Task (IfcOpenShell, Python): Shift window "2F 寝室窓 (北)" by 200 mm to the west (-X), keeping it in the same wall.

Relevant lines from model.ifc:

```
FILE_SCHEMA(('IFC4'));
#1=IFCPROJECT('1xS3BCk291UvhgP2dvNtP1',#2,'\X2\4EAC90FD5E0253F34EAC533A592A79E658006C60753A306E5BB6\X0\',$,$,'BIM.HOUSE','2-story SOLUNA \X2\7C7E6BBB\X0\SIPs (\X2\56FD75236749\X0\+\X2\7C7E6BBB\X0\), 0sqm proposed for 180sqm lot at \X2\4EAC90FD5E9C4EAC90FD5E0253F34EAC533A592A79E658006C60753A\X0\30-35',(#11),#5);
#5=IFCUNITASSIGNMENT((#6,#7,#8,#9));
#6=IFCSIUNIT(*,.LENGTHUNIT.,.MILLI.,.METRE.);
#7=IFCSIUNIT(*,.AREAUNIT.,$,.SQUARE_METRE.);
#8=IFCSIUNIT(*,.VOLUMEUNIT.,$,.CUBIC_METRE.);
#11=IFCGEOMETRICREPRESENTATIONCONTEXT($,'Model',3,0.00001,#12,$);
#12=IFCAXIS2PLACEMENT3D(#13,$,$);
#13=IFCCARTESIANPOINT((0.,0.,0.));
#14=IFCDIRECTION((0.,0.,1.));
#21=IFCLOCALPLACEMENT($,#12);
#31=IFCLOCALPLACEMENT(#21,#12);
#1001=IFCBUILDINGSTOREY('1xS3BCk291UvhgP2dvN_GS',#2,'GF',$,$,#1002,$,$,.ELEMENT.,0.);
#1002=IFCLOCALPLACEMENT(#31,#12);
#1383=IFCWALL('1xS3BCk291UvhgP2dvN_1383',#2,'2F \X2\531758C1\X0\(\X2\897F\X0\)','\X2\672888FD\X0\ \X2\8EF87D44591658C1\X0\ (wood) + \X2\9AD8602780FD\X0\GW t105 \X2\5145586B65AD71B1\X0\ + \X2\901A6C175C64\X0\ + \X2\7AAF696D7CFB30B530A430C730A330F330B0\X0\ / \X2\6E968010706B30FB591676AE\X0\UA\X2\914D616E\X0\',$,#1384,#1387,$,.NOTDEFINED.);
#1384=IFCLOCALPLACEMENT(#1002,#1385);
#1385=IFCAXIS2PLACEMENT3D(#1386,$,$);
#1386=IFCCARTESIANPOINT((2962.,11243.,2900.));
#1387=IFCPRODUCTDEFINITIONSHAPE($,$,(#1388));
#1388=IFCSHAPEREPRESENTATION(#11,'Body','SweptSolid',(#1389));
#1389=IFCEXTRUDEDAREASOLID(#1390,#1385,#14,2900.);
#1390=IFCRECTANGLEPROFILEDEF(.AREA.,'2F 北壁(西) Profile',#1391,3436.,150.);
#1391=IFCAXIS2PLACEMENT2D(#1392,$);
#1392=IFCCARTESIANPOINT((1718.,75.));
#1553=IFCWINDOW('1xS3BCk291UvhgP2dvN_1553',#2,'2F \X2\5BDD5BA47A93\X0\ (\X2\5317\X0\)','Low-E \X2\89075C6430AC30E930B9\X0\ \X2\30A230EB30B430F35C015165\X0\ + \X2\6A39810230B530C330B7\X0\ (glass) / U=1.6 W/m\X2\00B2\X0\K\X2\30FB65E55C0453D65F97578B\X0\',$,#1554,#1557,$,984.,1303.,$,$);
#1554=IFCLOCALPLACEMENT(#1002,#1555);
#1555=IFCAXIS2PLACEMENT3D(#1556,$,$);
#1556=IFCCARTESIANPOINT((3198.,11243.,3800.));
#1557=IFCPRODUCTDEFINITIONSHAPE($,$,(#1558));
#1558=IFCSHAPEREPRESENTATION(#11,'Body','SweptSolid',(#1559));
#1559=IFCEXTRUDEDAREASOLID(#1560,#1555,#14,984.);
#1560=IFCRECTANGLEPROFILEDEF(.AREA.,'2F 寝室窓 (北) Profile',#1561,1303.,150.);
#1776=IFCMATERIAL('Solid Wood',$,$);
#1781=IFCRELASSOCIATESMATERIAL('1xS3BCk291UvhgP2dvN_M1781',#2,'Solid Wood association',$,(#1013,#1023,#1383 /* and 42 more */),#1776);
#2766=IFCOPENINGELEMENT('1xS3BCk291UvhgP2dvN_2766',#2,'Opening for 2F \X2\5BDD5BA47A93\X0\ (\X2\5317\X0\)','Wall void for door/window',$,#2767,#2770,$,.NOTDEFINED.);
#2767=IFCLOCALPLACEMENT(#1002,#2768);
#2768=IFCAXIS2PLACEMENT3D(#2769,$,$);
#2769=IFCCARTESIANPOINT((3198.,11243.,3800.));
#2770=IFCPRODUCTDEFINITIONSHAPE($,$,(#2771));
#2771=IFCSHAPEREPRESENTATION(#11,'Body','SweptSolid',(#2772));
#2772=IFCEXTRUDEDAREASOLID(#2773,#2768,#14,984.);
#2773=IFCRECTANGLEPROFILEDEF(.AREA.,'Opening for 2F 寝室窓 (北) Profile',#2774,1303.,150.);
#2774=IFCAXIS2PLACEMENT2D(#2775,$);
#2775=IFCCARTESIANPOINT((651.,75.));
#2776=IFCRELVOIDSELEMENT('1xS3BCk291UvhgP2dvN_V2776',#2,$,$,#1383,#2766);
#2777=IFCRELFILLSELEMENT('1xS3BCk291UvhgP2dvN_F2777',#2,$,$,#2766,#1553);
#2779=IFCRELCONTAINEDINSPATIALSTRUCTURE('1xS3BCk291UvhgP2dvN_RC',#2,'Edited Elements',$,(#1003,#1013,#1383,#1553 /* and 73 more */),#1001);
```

```python
import ifcopenshell
import ifcopenshell.api.geometry
import ifcopenshell.util.placement
import ifcopenshell.util.unit

model = ifcopenshell.open("model.ifc")
unit_scale = ifcopenshell.util.unit.calculate_unit_scale(model)

window = model.by_id(1553)
opening = window.FillsVoids[0].RelatingOpeningElement
wall = opening.VoidsElements[0].RelatingBuildingElement

wall_matrix = ifcopenshell.util.placement.get_local_placement(wall.ObjectPlacement)
shift = wall_matrix[:3, 0] * -0.2 / unit_scale
before = ifcopenshell.util.placement.get_local_placement(window.ObjectPlacement)[:3, 3].copy()

# The window is not placed relative to its opening, so move both.
for product in (opening, window):
    matrix = ifcopenshell.util.placement.get_local_placement(product.ObjectPlacement)
    matrix[:3, 3] += shift
    ifcopenshell.api.geometry.edit_object_placement(model, product=product, matrix=matrix, is_si=False)

after = ifcopenshell.util.placement.get_local_placement(window.ObjectPlacement)[:3, 3]
print("window moved by", (after - before).round(3) + 0.0)

model.write("model_v2.ifc")
```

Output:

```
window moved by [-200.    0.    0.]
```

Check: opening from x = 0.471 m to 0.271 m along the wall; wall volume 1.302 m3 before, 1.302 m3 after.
